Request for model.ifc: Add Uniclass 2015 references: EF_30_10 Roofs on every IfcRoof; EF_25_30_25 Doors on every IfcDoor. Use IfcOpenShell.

First a look at what the model holds.

```python
import ifcopenshell

model = ifcopenshell.open("model.ifc")
print(model.schema)
print("classifications:", [c.Name for c in model.by_type("IfcClassification")])
for ifc_class in ("IfcDoor", "IfcRoof", "IfcStair", "IfcWall", "IfcWindow"):
    print(ifc_class, len(model.by_type(ifc_class)))
```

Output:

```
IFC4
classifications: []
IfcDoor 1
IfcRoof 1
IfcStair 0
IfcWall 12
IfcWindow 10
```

```python
import ifcopenshell
import ifcopenshell.api.classification

model = ifcopenshell.open("model.ifc")

system = ifcopenshell.api.classification.add_classification(model, classification="Uniclass 2015")

codes = {
    "IfcRoof": ("EF_30_10", "Roofs"),
    "IfcDoor": ("EF_25_30_25", "Doors"),
}
for ifc_class, (code, name) in codes.items():
    products = model.by_type(ifc_class)
    ifcopenshell.api.classification.add_reference(
        model, products=products, classification=system, identification=code, name=name
    )
    print(code, len(products))

model.write("model_updated.ifc")
```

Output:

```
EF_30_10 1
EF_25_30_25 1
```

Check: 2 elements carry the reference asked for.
